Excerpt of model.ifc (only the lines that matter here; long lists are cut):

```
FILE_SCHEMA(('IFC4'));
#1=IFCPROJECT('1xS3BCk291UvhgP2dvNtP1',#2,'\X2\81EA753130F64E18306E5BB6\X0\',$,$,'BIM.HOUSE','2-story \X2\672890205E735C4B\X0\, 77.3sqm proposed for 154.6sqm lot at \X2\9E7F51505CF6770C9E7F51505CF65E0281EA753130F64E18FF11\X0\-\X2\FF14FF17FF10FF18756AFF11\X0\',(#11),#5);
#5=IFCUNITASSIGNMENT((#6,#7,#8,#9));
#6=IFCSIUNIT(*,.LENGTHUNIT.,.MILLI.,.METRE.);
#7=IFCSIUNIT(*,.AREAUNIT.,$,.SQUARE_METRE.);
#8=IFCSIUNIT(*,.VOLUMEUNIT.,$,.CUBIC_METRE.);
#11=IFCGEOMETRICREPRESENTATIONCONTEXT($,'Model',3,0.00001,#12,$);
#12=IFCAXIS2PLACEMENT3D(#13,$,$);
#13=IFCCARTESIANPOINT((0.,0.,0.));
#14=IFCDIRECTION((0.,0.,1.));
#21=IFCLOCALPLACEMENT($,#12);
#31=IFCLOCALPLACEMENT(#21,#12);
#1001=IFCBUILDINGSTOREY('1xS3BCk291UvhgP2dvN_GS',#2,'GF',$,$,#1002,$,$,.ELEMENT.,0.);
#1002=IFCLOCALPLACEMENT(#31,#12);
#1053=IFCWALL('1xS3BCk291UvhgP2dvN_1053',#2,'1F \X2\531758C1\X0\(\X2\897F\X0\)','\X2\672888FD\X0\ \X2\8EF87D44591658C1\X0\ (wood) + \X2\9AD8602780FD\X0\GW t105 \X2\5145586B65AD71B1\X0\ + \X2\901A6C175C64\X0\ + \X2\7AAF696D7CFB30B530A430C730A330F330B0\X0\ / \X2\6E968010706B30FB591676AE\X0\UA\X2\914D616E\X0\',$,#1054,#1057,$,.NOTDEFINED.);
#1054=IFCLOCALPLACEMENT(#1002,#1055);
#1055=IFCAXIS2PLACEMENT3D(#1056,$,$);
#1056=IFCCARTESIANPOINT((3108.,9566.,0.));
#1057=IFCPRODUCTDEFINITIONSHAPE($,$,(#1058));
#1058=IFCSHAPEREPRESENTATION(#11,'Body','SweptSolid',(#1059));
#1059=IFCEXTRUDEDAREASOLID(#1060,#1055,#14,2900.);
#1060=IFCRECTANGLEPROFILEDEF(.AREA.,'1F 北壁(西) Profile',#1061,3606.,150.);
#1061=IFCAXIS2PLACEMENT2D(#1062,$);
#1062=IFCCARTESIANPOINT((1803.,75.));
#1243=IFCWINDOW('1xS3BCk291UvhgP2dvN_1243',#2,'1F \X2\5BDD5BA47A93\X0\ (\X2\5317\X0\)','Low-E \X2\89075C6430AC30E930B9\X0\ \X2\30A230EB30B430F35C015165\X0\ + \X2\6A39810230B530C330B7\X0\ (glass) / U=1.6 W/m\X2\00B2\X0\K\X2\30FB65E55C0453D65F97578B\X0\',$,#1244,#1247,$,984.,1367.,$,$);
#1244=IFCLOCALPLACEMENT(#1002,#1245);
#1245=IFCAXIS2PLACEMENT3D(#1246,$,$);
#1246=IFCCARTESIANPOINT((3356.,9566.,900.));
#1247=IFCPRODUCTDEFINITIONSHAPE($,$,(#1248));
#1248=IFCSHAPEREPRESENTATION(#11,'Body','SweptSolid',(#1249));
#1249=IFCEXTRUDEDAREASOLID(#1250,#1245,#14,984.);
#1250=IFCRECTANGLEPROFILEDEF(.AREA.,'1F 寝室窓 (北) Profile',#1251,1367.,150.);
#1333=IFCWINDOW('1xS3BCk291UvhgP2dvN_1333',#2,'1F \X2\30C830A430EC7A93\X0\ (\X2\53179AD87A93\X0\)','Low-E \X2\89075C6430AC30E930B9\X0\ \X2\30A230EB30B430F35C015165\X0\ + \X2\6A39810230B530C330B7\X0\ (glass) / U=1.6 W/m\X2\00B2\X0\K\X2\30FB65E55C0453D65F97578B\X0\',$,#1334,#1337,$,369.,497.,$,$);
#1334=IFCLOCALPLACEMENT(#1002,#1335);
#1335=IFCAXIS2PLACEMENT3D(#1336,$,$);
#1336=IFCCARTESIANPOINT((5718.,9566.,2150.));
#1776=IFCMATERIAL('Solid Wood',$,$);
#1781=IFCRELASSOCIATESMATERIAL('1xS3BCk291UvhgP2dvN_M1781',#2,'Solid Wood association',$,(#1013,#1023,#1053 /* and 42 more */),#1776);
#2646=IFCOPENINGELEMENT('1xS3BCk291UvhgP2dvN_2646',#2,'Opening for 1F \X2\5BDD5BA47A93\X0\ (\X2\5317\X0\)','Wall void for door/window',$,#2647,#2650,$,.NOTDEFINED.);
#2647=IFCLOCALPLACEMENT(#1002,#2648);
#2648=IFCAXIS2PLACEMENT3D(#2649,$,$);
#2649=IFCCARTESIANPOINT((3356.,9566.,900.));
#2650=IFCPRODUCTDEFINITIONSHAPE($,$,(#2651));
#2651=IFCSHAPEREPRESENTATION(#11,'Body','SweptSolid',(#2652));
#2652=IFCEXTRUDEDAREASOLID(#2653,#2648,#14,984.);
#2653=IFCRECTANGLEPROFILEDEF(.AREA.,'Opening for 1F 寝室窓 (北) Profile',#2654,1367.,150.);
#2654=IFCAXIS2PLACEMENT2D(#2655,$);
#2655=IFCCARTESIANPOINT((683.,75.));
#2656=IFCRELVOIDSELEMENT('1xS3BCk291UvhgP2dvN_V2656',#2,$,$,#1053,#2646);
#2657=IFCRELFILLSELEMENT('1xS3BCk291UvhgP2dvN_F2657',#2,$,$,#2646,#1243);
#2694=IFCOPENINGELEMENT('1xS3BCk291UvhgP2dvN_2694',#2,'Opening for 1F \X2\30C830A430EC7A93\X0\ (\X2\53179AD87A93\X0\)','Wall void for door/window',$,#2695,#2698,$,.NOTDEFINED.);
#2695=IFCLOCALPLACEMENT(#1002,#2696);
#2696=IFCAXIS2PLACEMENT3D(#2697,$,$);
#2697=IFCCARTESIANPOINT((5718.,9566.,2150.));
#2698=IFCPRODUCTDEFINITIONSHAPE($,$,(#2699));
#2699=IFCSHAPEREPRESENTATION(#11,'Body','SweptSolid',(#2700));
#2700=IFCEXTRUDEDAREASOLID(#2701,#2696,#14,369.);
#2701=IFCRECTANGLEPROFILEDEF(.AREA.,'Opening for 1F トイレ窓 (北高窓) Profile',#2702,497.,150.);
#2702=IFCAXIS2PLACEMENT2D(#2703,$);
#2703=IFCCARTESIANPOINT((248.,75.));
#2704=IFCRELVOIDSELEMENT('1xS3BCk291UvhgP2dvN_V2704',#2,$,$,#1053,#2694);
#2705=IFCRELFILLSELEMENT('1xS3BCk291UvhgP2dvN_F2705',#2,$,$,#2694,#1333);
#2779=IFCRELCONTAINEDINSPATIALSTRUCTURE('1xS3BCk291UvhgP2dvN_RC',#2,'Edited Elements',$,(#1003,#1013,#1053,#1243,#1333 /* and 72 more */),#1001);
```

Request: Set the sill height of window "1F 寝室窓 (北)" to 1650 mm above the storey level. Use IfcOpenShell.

```python
import numpy as np
import ifcopenshell
import ifcopenshell.api.geometry
import ifcopenshell.geom
import ifcopenshell.util.element
import ifcopenshell.util.placement
import ifcopenshell.util.shape
import ifcopenshell.util.unit

model = ifcopenshell.open("model.ifc")
unit_scale = ifcopenshell.util.unit.calculate_unit_scale(model)

window = model.by_guid("1xS3BCk291UvhgP2dvN_1243")
opening = window.FillsVoids[0].RelatingOpeningElement
storey = ifcopenshell.util.element.get_container(window, ifc_class="IfcBuildingStorey")
level = ifcopenshell.util.placement.get_local_placement(storey.ObjectPlacement)[2, 3]

# The opening's origin need not be at the sill, so measure its lowest point.
shape = ifcopenshell.geom.create_shape(ifcopenshell.geom.settings(), opening)
bottom = ifcopenshell.util.shape.get_shape_bottom_elevation(shape, shape.geometry) / unit_scale
dz = level + 1650.0 - bottom

shift = np.array([0.0, 0.0, dz])
# The window is not placed relative to its opening, so move both.
for product in (opening, window):
    matrix = ifcopenshell.util.placement.get_local_placement(product.ObjectPlacement)
    matrix[:3, 3] += shift
    ifcopenshell.api.geometry.edit_object_placement(model, product=product, matrix=matrix, is_si=False)

print(f"moved by {dz * unit_scale:+.3f} m")

model.write("model_edited.ifc")
```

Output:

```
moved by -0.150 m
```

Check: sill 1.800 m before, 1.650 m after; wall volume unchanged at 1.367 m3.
